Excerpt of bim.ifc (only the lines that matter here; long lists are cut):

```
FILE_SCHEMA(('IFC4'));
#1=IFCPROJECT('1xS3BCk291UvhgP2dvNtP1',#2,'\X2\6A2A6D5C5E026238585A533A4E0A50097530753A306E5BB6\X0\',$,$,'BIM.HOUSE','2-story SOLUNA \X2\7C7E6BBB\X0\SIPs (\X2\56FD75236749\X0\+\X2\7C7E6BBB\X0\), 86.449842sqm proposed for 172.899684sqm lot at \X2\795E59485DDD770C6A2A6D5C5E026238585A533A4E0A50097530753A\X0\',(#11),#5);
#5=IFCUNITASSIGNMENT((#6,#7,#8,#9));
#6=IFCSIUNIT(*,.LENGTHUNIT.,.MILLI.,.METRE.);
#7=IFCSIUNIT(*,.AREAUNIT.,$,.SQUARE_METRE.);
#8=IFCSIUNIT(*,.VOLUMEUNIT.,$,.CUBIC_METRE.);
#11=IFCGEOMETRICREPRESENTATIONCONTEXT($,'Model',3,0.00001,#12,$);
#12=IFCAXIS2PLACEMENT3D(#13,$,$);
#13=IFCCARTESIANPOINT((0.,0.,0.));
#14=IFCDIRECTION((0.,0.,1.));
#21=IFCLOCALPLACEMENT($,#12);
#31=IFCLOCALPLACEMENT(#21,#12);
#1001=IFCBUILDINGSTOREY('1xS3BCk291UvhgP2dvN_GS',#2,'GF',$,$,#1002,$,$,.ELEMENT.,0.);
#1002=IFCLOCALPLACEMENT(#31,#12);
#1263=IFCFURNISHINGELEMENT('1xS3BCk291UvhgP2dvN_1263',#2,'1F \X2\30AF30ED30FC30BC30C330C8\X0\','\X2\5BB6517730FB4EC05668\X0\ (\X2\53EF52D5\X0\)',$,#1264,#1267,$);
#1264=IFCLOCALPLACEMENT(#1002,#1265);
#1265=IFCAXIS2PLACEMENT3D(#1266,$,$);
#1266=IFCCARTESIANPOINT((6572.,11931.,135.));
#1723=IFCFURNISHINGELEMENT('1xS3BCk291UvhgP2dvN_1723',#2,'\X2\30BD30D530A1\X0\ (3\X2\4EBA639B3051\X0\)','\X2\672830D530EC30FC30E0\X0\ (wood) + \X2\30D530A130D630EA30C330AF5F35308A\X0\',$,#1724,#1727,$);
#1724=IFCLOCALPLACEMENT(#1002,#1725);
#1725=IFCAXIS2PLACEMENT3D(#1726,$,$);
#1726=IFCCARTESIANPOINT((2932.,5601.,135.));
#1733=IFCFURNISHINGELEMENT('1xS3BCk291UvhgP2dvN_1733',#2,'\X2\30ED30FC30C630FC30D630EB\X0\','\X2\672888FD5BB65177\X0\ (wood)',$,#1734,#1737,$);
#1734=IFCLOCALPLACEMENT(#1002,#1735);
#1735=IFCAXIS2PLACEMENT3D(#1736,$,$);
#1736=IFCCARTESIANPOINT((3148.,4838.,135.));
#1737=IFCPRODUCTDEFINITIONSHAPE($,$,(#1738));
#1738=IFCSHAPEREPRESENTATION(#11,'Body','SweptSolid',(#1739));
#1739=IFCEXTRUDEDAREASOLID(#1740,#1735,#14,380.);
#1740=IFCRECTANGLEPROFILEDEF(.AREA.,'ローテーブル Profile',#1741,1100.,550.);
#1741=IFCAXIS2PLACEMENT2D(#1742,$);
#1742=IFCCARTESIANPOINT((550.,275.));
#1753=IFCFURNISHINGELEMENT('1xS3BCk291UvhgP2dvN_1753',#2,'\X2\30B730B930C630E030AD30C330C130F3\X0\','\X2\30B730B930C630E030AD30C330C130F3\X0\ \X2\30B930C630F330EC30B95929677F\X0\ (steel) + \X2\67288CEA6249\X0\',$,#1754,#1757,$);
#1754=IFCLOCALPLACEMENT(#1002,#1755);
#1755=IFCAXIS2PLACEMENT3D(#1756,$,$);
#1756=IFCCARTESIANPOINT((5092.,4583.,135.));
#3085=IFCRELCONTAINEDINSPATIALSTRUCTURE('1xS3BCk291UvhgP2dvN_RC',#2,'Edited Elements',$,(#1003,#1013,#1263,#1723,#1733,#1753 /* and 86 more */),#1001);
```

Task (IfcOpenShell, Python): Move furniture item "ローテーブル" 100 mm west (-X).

```python
import ifcopenshell
import ifcopenshell.api.geometry
import ifcopenshell.util.placement
import ifcopenshell.util.unit

model = ifcopenshell.open("bim.ifc")
unit_scale = ifcopenshell.util.unit.calculate_unit_scale(model)

item = model.by_id(1733)
matrix = ifcopenshell.util.placement.get_local_placement(item.ObjectPlacement)
matrix[0, 3] -= 0.1 / unit_scale
ifcopenshell.api.geometry.edit_object_placement(model, product=item, matrix=matrix, is_si=False)

print(ifcopenshell.util.placement.get_local_placement(item.ObjectPlacement).round(3) + 0.0)

model.write("bim_v2.ifc")
```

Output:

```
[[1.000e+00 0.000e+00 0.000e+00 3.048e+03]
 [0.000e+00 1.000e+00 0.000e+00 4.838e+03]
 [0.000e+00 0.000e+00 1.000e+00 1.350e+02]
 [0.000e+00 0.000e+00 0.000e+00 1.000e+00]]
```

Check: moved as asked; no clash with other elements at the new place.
